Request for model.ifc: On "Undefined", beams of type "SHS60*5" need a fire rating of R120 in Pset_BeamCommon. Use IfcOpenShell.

First a look at what the model holds.

```python
import ifcopenshell
import ifcopenshell.util.element

model = ifcopenshell.open("model.ifc")
print(model.schema)
storey = next(s for s in model.by_type("IfcBuildingStorey") if s.Name == "Undefined")
beams = [e for e in ifcopenshell.util.element.get_decomposition(storey) if e.is_a("IfcBeam")]
seen = {}
for e in beams:
    element_type = ifcopenshell.util.element.get_type(e)
    key = (element_type.Name if element_type != e and element_type else None, ifcopenshell.util.element.get_pset(e, "Pset_BeamCommon", "FireRating"))
    seen[key] = seen.get(key, 0) + 1
for (name, value), count in sorted(seen.items(), key=str):
    print(count, "x", name, "|", value)
```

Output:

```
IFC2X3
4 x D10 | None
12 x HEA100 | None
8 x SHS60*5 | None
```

```python
import ifcopenshell
import ifcopenshell.api.pset
import ifcopenshell.util.element

model = ifcopenshell.open("model.ifc")

storey = next(s for s in model.by_type("IfcBuildingStorey") if s.Name == "Undefined")
beams = [e for e in ifcopenshell.util.element.get_decomposition(storey) if e.is_a("IfcBeam")]

count = 0
for e in beams:
    element_type = ifcopenshell.util.element.get_type(e)
    if element_type in (None, e) or element_type.Name != "SHS60*5":
        continue
    # add_pset returns the element's existing set when there is one.
    pset = ifcopenshell.api.pset.add_pset(model, product=e, name="Pset_BeamCommon")
    ifcopenshell.api.pset.edit_pset(model, pset=pset, properties={"FireRating": "R120"})
    count += 1

print(count, "beams updated")

model.write("model_rev.ifc")
```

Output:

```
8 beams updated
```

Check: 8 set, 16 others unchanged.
